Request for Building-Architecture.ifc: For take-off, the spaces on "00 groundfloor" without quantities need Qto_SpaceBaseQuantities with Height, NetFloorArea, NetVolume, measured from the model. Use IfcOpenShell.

First a look at what the model holds.

```python
import ifcopenshell
import ifcopenshell.util.element
import ifcopenshell.util.unit

model = ifcopenshell.open("Building-Architecture.ifc")
print(model.schema)
for unit_type in ("LENGTHUNIT", "AREAUNIT", "VOLUMEUNIT"):
    print(unit_type, ifcopenshell.util.unit.calculate_unit_scale(model, unit_type))
storey = next(s for s in model.by_type("IfcBuildingStorey") if s.Name == "00 groundfloor")
spaces = [e for e in ifcopenshell.util.element.get_decomposition(storey) if e.is_a("IfcSpace")]
for e in sorted(spaces, key=lambda e: e.id()):
    print(e.id(), e.is_a(), e.Name, list(ifcopenshell.util.element.get_psets(e, qtos_only=True)), sep=" | ")
```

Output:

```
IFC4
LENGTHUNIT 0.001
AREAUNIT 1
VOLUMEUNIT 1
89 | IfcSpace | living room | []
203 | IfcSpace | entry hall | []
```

```python
import ifcopenshell
import ifcopenshell.api.pset
import ifcopenshell.geom
import ifcopenshell.util.element
import ifcopenshell.util.shape
import ifcopenshell.util.unit

model = ifcopenshell.open("Building-Architecture.ifc")
unit_scale = ifcopenshell.util.unit.calculate_unit_scale(model)
area_scale = ifcopenshell.util.unit.calculate_unit_scale(model, "AREAUNIT")
volume_scale = ifcopenshell.util.unit.calculate_unit_scale(model, "VOLUMEUNIT")
settings = ifcopenshell.geom.settings()

storey = next(s for s in model.by_type("IfcBuildingStorey") if s.Name == "00 groundfloor")
spaces = [e for e in ifcopenshell.util.element.get_decomposition(storey) if e.is_a("IfcSpace")]

for e in sorted(spaces, key=lambda e: e.id()):
    if ifcopenshell.util.element.get_psets(e, qtos_only=True, should_inherit=False):
        continue
    # Geometry comes back in metres, in the element's own axes.
    shape = ifcopenshell.geom.create_shape(settings, e)
    values = {
        "Height": ifcopenshell.util.shape.get_z(shape.geometry) / unit_scale,
        "NetFloorArea": ifcopenshell.util.shape.get_footprint_area(shape.geometry) / area_scale,
        "NetVolume": ifcopenshell.util.shape.get_volume(shape.geometry) / volume_scale,
    }
    qto = ifcopenshell.api.pset.add_qto(model, product=e, name="Qto_SpaceBaseQuantities")
    ifcopenshell.api.pset.edit_qto(model, qto=qto, properties=values)
    print(e.id(), {k: round(v, 3) for k, v in values.items()})

model.write("Building-Architecture_v2.ifc")
```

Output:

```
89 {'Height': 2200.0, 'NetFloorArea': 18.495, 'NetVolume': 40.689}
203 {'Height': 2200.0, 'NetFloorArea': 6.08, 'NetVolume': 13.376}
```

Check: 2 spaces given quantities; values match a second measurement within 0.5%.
